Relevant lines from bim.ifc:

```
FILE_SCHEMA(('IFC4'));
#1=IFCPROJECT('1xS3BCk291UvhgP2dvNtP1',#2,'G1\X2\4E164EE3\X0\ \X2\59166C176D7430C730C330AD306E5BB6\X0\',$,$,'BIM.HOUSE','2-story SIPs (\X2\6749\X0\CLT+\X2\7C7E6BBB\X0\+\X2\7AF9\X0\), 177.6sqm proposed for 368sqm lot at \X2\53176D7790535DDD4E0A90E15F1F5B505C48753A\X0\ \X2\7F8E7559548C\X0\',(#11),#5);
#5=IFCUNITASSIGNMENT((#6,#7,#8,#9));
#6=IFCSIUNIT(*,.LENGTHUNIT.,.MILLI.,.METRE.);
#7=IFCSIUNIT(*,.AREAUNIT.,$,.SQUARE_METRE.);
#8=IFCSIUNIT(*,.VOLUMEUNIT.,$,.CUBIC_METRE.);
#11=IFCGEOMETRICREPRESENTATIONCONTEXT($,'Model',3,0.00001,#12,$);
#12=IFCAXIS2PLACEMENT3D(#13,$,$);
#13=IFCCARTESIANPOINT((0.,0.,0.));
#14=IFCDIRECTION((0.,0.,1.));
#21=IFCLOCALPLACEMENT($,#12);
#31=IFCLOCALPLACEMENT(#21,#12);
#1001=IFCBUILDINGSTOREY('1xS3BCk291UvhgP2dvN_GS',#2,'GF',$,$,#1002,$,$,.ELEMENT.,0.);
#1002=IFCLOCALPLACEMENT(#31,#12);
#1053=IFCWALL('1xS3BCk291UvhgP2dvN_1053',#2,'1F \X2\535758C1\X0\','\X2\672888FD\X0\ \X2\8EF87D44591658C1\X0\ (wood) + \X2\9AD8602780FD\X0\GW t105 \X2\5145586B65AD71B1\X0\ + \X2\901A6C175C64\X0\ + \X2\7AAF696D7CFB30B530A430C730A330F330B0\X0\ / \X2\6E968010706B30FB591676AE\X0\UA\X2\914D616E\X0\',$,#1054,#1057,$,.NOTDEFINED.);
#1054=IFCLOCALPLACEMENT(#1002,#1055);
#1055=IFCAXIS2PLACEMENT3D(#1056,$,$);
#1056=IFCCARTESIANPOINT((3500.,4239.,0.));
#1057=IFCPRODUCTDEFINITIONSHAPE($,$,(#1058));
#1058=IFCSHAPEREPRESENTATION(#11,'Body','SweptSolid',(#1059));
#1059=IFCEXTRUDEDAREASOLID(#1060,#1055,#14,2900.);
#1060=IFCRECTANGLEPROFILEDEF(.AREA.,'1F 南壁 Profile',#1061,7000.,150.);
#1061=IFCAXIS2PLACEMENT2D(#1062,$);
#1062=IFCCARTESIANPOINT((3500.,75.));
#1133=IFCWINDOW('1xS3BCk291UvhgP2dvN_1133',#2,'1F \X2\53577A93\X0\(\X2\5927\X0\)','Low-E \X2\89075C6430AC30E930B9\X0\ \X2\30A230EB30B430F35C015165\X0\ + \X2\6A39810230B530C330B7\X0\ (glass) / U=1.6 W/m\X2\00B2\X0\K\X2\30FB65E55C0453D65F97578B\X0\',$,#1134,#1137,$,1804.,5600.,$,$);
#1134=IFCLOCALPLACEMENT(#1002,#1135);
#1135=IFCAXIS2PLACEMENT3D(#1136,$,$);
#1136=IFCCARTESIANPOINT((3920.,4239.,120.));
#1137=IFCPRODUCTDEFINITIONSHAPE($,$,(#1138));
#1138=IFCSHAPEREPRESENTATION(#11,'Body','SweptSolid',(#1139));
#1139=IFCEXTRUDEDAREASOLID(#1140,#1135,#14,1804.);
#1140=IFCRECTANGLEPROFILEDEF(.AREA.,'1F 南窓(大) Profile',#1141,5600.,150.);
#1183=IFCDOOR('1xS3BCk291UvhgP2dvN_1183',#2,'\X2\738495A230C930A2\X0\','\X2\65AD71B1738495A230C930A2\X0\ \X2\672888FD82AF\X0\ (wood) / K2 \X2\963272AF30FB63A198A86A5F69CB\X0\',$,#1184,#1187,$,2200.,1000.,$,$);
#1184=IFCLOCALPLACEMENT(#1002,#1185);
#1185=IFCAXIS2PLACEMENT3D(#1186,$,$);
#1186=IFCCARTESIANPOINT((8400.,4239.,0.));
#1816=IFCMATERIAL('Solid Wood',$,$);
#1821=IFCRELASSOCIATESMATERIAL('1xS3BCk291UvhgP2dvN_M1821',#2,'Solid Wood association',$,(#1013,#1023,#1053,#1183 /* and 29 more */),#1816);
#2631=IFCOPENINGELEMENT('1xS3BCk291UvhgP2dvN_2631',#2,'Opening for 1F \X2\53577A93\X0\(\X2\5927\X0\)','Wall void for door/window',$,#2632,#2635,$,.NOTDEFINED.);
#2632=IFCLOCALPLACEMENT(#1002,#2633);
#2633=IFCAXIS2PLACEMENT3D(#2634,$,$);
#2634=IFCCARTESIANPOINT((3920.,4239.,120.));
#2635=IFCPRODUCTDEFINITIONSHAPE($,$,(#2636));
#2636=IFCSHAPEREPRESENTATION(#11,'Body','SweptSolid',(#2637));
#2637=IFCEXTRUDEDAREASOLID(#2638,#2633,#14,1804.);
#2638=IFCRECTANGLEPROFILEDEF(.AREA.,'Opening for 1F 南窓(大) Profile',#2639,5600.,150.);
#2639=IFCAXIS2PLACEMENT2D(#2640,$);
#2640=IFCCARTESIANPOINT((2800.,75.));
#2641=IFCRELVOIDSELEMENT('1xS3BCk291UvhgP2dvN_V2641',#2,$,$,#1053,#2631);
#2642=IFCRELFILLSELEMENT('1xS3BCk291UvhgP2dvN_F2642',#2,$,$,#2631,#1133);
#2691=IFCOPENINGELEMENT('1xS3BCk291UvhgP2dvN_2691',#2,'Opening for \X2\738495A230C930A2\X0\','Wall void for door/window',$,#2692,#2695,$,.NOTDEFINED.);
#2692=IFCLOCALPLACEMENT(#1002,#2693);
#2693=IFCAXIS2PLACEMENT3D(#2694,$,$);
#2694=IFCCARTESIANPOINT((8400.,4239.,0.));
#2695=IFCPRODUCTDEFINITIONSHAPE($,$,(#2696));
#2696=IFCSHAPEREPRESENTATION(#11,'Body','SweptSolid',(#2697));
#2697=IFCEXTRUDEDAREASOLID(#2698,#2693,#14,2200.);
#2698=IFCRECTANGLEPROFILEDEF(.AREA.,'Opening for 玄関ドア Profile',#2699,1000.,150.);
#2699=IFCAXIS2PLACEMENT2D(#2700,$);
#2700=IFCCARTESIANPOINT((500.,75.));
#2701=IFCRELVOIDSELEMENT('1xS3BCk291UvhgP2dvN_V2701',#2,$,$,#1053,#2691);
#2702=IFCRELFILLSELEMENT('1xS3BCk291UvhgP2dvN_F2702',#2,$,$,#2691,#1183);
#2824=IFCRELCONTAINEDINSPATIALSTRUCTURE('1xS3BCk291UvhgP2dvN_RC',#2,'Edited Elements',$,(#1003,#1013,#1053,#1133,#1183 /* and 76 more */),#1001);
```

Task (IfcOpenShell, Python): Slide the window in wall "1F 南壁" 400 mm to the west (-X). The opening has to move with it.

```python
import ifcopenshell
import ifcopenshell.api.geometry
import ifcopenshell.util.placement

model = ifcopenshell.open("bim.ifc")

window = model.by_guid("1xS3BCk291UvhgP2dvN_1133")
opening = window.FillsVoids[0].RelatingOpeningElement
wall = opening.VoidsElements[0].RelatingBuildingElement

wall_matrix = ifcopenshell.util.placement.get_local_placement(wall.ObjectPlacement)
shift = wall_matrix[:3, 0] * -400.0
before = ifcopenshell.util.placement.get_local_placement(window.ObjectPlacement)[:3, 3].copy()

# The window is not placed relative to its opening, so move both.
for product in (opening, window):
    matrix = ifcopenshell.util.placement.get_local_placement(product.ObjectPlacement)
    matrix[:3, 3] += shift
    ifcopenshell.api.geometry.edit_object_placement(model, product=product, matrix=matrix, is_si=False)

after = ifcopenshell.util.placement.get_local_placement(window.ObjectPlacement)[:3, 3]
print("window moved by", (after - before).round(3) + 0.0)

model.write("bim_updated.ifc")
```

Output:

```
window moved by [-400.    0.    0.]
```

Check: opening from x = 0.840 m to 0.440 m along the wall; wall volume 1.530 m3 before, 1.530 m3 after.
